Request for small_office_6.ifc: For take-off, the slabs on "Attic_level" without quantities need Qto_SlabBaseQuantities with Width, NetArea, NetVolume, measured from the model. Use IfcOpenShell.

First a look at what the model holds.

```python
import ifcopenshell
import ifcopenshell.util.element
import ifcopenshell.util.unit

model = ifcopenshell.open("small_office_6.ifc")
print(model.schema)
for unit_type in ("LENGTHUNIT", "AREAUNIT", "VOLUMEUNIT"):
    print(unit_type, ifcopenshell.util.unit.calculate_unit_scale(model, unit_type))
storey = next(s for s in model.by_type("IfcBuildingStorey") if s.Name == "Attic_level")
slabs = [e for e in ifcopenshell.util.element.get_decomposition(storey) if e.is_a("IfcSlab")]
for e in sorted(slabs, key=lambda e: e.id()):
    print(e.id(), e.is_a(), e.Name, list(ifcopenshell.util.element.get_psets(e, qtos_only=True)), sep=" | ")
```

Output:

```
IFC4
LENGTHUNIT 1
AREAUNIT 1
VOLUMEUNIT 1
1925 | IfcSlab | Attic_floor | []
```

```python
import ifcopenshell
import ifcopenshell.api.pset
import ifcopenshell.geom
import ifcopenshell.util.element
import ifcopenshell.util.shape
import ifcopenshell.util.unit

model = ifcopenshell.open("small_office_6.ifc")
unit_scale = ifcopenshell.util.unit.calculate_unit_scale(model)
area_scale = ifcopenshell.util.unit.calculate_unit_scale(model, "AREAUNIT")
volume_scale = ifcopenshell.util.unit.calculate_unit_scale(model, "VOLUMEUNIT")
settings = ifcopenshell.geom.settings()

storey = next(s for s in model.by_type("IfcBuildingStorey") if s.Name == "Attic_level")
slabs = [e for e in ifcopenshell.util.element.get_decomposition(storey) if e.is_a("IfcSlab")]

for e in sorted(slabs, key=lambda e: e.id()):
    if ifcopenshell.util.element.get_psets(e, qtos_only=True, should_inherit=False):
        continue
    # Geometry comes back in metres, in the element's own axes.
    shape = ifcopenshell.geom.create_shape(settings, e)
    values = {
        "Width": ifcopenshell.util.shape.get_z(shape.geometry) / unit_scale,
        "NetArea": ifcopenshell.util.shape.get_footprint_area(shape.geometry) / area_scale,
        "NetVolume": ifcopenshell.util.shape.get_volume(shape.geometry) / volume_scale,
    }
    qto = ifcopenshell.api.pset.add_qto(model, product=e, name="Qto_SlabBaseQuantities")
    ifcopenshell.api.pset.edit_qto(model, qto=qto, properties=values)
    print(e.id(), {k: round(v, 3) for k, v in values.items()})

model.write("small_office_6_rev.ifc")
```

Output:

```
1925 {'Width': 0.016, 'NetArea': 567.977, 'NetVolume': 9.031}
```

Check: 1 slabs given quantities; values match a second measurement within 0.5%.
